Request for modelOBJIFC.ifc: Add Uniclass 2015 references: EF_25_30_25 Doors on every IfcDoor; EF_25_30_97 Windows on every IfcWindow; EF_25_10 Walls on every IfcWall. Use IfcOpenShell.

First a look at what the model holds.

```python
import ifcopenshell

model = ifcopenshell.open("modelOBJIFC.ifc")
print(model.schema)
print("classifications:", [c.Name for c in model.by_type("IfcClassification")])
for ifc_class in ("IfcDoor", "IfcRoof", "IfcStair", "IfcWall", "IfcWindow"):
    print(ifc_class, len(model.by_type(ifc_class)))
```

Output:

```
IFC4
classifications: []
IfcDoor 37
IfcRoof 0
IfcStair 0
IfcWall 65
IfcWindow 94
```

```python
import ifcopenshell
import ifcopenshell.api.classification

model = ifcopenshell.open("modelOBJIFC.ifc")

system = ifcopenshell.api.classification.add_classification(model, classification="Uniclass 2015")

codes = {
    "IfcDoor": ("EF_25_30_25", "Doors"),
    "IfcWindow": ("EF_25_30_97", "Windows"),
    "IfcWall": ("EF_25_10", "Walls"),
}
for ifc_class, (code, name) in codes.items():
    products = model.by_type(ifc_class)
    ifcopenshell.api.classification.add_reference(
        model, products=products, classification=system, identification=code, name=name
    )
    print(code, len(products))

model.write("modelOBJIFC_updated.ifc")
```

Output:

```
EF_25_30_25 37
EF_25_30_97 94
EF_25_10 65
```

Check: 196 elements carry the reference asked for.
